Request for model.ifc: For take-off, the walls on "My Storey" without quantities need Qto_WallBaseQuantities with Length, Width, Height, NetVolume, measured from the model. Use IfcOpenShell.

First a look at what the model holds.

```python
import ifcopenshell
import ifcopenshell.util.element
import ifcopenshell.util.unit

model = ifcopenshell.open("model.ifc")
print(model.schema)
for unit_type in ("LENGTHUNIT", "AREAUNIT", "VOLUMEUNIT"):
    print(unit_type, ifcopenshell.util.unit.calculate_unit_scale(model, unit_type))
storey = next(s for s in model.by_type("IfcBuildingStorey") if s.Name == "My Storey")
walls = [e for e in ifcopenshell.util.element.get_decomposition(storey) if e.is_a("IfcWall")]
for e in sorted(walls, key=lambda e: e.id()):
    print(e.id(), e.is_a(), e.Name, list(ifcopenshell.util.element.get_psets(e, qtos_only=True)), sep=" | ")
```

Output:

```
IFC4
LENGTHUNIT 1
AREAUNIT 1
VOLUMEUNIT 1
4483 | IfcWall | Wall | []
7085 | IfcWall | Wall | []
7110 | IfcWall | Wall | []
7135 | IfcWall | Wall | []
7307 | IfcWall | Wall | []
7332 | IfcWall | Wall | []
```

```python
import ifcopenshell
import ifcopenshell.api.pset
import ifcopenshell.geom
import ifcopenshell.util.element
import ifcopenshell.util.shape
import ifcopenshell.util.unit

model = ifcopenshell.open("model.ifc")
unit_scale = ifcopenshell.util.unit.calculate_unit_scale(model)
volume_scale = ifcopenshell.util.unit.calculate_unit_scale(model, "VOLUMEUNIT")
settings = ifcopenshell.geom.settings()

storey = next(s for s in model.by_type("IfcBuildingStorey") if s.Name == "My Storey")
walls = [e for e in ifcopenshell.util.element.get_decomposition(storey) if e.is_a("IfcWall")]

for e in sorted(walls, key=lambda e: e.id()):
    if ifcopenshell.util.element.get_psets(e, qtos_only=True, should_inherit=False):
        continue
    # Geometry comes back in metres, in the element's own axes.
    shape = ifcopenshell.geom.create_shape(settings, e)
    values = {
        "Length": ifcopenshell.util.shape.get_x(shape.geometry) / unit_scale,
        "Width": ifcopenshell.util.shape.get_y(shape.geometry) / unit_scale,
        "Height": ifcopenshell.util.shape.get_z(shape.geometry) / unit_scale,
        "NetVolume": ifcopenshell.util.shape.get_volume(shape.geometry) / volume_scale,
    }
    qto = ifcopenshell.api.pset.add_qto(model, product=e, name="Qto_WallBaseQuantities")
    ifcopenshell.api.pset.edit_qto(model, qto=qto, properties=values)
    print(e.id(), {k: round(v, 3) for k, v in values.items()})

model.write("model_updated.ifc")
```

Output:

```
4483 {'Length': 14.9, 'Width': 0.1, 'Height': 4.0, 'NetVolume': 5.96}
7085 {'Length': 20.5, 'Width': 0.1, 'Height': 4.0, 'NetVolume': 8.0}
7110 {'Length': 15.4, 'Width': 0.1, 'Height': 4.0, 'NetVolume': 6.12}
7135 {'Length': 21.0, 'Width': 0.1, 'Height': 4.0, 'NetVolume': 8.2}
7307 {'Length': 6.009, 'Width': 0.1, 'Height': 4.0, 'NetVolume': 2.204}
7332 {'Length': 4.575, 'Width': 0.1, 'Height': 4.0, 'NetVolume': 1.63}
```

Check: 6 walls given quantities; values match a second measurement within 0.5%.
